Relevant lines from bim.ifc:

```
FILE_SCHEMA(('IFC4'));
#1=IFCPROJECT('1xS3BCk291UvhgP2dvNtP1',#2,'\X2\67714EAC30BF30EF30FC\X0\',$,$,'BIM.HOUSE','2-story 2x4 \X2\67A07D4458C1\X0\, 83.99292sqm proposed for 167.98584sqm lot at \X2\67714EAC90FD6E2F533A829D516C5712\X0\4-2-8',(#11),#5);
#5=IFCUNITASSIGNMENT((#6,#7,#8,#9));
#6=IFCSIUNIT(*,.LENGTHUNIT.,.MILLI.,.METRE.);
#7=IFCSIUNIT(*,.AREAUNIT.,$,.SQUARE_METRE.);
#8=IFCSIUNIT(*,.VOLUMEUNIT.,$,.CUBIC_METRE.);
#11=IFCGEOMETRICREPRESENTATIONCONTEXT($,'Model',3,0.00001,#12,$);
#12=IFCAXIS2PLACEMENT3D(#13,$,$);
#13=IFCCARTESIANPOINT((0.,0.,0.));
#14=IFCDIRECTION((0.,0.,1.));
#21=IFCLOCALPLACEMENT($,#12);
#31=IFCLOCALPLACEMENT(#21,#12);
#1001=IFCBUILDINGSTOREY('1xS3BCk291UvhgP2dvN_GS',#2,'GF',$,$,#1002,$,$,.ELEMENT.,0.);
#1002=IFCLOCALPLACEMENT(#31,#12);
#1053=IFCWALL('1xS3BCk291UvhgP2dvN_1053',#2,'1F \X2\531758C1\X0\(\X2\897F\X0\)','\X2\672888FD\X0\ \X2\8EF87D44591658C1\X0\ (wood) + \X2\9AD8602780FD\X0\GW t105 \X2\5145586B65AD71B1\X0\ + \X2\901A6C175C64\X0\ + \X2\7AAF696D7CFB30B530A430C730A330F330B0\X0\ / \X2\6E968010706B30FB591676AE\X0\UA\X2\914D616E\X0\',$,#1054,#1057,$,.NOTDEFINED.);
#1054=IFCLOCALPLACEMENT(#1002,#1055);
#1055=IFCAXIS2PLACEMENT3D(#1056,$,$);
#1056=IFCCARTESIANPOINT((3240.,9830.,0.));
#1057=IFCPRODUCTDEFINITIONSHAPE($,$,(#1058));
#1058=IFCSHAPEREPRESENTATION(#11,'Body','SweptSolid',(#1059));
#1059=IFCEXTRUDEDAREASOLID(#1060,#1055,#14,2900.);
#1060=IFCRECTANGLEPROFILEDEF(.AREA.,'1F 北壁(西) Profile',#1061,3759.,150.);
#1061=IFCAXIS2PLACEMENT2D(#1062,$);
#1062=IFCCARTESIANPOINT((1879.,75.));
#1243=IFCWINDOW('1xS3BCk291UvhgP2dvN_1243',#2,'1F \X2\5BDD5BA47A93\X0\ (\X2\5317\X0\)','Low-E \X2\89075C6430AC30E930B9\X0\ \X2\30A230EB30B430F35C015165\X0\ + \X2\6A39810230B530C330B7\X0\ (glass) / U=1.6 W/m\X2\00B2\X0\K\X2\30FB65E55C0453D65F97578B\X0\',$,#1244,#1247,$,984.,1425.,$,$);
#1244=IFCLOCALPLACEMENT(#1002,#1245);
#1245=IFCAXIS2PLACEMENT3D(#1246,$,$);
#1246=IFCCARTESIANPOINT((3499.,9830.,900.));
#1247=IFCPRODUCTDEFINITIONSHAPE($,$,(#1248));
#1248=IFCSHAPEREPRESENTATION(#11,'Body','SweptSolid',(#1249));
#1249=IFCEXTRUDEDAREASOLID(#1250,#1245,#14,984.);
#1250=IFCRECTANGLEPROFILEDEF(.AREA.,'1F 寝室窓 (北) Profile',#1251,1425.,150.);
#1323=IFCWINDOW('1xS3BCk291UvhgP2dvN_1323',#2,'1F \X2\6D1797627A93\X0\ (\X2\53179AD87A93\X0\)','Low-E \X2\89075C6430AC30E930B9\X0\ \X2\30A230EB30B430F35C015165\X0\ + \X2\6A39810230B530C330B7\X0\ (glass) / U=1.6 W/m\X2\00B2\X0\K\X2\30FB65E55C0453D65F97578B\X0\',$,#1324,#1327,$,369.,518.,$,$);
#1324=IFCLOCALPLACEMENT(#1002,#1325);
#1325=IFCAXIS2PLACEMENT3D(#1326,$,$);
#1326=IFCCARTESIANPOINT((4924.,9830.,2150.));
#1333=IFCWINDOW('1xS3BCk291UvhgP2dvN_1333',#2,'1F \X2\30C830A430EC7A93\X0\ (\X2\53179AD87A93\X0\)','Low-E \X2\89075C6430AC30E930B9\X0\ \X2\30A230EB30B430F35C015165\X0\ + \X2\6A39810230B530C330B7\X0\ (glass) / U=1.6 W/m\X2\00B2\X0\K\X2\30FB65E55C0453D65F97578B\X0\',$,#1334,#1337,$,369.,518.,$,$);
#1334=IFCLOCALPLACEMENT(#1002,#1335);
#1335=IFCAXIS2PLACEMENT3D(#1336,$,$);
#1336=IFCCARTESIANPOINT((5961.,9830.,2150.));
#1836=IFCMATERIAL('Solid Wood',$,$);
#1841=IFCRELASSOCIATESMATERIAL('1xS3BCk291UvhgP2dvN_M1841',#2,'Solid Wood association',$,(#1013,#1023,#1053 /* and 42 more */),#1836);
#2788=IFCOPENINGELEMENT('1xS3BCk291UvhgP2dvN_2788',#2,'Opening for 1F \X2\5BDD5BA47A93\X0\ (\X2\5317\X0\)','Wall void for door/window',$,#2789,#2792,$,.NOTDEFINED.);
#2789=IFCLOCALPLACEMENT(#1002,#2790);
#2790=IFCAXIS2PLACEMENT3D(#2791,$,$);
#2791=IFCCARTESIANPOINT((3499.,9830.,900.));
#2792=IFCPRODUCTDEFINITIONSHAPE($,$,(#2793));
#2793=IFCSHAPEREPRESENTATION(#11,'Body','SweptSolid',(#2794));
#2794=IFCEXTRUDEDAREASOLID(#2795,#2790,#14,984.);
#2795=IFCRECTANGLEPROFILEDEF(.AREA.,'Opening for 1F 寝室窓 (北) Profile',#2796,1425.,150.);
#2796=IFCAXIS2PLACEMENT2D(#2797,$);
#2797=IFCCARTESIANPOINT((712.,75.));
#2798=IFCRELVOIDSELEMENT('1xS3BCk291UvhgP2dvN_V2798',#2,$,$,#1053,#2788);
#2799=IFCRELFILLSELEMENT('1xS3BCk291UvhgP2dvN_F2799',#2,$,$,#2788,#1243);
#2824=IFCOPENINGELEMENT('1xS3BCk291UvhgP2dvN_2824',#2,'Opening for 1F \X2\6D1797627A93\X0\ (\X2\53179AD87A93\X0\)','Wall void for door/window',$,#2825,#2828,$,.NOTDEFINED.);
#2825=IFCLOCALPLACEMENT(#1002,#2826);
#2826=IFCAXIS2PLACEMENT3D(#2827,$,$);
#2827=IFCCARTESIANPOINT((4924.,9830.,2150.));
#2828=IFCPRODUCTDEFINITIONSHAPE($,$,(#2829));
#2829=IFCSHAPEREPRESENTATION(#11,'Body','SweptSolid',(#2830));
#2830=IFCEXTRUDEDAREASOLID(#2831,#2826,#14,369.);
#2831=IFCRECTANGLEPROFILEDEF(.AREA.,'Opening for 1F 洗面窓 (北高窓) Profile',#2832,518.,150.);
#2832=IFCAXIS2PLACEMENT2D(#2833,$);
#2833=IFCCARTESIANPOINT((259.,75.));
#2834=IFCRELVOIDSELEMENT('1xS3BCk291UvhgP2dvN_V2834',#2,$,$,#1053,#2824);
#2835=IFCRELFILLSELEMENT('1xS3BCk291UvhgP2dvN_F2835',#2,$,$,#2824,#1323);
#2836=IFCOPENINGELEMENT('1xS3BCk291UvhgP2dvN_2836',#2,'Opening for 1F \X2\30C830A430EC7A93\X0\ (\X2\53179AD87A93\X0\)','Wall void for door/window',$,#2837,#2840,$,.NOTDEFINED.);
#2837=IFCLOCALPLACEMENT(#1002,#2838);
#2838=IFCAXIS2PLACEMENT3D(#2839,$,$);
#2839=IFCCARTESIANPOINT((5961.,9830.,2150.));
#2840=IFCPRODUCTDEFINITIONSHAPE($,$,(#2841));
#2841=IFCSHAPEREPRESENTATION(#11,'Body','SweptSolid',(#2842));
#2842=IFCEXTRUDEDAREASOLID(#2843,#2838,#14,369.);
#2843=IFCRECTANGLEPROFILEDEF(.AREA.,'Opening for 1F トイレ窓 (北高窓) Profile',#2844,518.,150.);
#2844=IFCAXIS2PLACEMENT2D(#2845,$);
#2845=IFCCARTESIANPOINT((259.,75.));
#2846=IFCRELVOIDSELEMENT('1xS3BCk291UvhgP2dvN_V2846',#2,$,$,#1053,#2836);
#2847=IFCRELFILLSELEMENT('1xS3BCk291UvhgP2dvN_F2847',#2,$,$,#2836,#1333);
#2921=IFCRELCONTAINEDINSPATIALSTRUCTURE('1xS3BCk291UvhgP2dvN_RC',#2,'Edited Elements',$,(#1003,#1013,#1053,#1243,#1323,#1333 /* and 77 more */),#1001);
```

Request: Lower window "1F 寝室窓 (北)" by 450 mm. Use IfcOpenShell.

```python
import numpy as np
import ifcopenshell
import ifcopenshell.api.geometry
import ifcopenshell.util.placement
import ifcopenshell.util.unit

model = ifcopenshell.open("bim.ifc")
unit_scale = ifcopenshell.util.unit.calculate_unit_scale(model)

window = model.by_id(1243)
opening = window.FillsVoids[0].RelatingOpeningElement
dz = -450.0

shift = np.array([0.0, 0.0, dz])
# The window is not placed relative to its opening, so move both.
for product in (opening, window):
    matrix = ifcopenshell.util.placement.get_local_placement(product.ObjectPlacement)
    matrix[:3, 3] += shift
    ifcopenshell.api.geometry.edit_object_placement(model, product=product, matrix=matrix, is_si=False)

print(f"moved by {dz * unit_scale:+.3f} m")

model.write("bim_v2.ifc")
```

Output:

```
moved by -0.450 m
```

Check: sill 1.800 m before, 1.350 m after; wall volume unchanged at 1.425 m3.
